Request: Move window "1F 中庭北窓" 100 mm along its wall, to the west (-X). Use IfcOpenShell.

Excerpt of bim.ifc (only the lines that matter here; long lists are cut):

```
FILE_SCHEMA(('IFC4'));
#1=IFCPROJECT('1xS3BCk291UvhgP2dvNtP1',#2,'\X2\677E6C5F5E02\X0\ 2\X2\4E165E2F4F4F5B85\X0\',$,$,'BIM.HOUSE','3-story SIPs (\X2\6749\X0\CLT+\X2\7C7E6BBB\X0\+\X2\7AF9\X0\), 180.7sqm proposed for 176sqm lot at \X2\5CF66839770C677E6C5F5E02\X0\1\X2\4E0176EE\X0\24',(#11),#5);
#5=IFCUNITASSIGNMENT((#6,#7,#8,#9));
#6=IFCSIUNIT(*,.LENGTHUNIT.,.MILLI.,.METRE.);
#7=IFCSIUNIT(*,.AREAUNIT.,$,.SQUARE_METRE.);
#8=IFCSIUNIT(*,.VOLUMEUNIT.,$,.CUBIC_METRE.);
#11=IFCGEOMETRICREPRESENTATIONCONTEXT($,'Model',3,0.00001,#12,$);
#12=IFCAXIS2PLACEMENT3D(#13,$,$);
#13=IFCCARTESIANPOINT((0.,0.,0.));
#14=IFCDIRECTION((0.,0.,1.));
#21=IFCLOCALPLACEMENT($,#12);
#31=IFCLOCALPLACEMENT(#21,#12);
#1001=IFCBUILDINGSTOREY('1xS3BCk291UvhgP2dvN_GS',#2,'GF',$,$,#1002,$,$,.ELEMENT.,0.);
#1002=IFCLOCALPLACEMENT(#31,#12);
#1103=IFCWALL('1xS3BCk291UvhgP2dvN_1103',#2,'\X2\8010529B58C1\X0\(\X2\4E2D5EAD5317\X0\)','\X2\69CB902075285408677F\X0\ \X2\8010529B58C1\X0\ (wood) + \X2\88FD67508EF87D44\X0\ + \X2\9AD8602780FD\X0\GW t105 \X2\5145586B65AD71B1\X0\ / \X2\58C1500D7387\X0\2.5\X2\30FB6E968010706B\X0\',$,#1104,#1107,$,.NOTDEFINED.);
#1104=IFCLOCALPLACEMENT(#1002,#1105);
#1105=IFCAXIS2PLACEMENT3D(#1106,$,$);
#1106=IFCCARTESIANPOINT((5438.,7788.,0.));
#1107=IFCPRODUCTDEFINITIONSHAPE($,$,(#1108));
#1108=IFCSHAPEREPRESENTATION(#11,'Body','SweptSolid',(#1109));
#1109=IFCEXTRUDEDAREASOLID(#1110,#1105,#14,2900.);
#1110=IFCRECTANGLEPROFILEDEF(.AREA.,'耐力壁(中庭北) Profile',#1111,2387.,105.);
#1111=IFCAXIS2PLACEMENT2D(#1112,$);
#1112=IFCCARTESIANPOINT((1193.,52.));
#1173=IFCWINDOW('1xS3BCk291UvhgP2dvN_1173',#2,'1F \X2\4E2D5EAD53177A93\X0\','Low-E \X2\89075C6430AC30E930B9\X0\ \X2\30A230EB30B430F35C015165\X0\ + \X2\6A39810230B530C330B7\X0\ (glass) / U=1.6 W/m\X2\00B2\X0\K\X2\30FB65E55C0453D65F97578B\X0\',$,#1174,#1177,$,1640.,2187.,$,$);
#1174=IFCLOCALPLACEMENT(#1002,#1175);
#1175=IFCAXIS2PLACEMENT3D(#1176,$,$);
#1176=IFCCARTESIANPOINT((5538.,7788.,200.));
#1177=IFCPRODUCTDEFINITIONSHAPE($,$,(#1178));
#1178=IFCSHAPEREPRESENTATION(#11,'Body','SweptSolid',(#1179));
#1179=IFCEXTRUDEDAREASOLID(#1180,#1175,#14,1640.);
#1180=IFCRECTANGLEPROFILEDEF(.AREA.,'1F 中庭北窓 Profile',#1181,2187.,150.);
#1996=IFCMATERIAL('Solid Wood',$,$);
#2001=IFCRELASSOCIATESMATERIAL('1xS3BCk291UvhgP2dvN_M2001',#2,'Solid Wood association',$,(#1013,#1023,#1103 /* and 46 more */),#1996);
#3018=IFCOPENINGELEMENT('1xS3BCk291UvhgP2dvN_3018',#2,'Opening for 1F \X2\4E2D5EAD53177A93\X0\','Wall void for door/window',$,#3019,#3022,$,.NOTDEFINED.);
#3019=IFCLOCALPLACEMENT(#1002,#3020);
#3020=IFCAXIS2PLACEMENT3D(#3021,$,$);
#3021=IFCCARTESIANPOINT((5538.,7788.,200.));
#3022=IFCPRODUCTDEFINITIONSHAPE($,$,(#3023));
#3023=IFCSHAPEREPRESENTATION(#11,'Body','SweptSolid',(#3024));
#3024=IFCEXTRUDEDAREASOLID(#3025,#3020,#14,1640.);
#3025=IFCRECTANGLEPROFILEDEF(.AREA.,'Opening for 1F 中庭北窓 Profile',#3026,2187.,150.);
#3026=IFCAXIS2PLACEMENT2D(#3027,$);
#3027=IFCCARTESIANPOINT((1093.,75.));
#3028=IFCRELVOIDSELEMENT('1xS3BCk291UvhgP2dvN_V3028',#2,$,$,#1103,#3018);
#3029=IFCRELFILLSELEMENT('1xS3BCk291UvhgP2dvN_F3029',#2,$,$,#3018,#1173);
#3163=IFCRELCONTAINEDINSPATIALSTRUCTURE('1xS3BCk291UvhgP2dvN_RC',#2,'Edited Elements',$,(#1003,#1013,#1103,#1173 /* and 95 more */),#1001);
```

```python
import ifcopenshell
import ifcopenshell.api.geometry
import ifcopenshell.util.placement

model = ifcopenshell.open("bim.ifc")

window = model.by_id(1173)
opening = window.FillsVoids[0].RelatingOpeningElement
wall = opening.VoidsElements[0].RelatingBuildingElement

wall_matrix = ifcopenshell.util.placement.get_local_placement(wall.ObjectPlacement)
shift = wall_matrix[:3, 0] * -100.0
before = ifcopenshell.util.placement.get_local_placement(window.ObjectPlacement)[:3, 3].copy()

# The window is not placed relative to its opening, so move both.
for product in (opening, window):
    matrix = ifcopenshell.util.placement.get_local_placement(product.ObjectPlacement)
    matrix[:3, 3] += shift
    ifcopenshell.api.geometry.edit_object_placement(model, product=product, matrix=matrix, is_si=False)

after = ifcopenshell.util.placement.get_local_placement(window.ObjectPlacement)[:3, 3]
print("window moved by", (after - before).round(3) + 0.0)

model.write("bim-out.ifc")
```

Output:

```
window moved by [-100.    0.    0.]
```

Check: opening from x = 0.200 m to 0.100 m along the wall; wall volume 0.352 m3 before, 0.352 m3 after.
